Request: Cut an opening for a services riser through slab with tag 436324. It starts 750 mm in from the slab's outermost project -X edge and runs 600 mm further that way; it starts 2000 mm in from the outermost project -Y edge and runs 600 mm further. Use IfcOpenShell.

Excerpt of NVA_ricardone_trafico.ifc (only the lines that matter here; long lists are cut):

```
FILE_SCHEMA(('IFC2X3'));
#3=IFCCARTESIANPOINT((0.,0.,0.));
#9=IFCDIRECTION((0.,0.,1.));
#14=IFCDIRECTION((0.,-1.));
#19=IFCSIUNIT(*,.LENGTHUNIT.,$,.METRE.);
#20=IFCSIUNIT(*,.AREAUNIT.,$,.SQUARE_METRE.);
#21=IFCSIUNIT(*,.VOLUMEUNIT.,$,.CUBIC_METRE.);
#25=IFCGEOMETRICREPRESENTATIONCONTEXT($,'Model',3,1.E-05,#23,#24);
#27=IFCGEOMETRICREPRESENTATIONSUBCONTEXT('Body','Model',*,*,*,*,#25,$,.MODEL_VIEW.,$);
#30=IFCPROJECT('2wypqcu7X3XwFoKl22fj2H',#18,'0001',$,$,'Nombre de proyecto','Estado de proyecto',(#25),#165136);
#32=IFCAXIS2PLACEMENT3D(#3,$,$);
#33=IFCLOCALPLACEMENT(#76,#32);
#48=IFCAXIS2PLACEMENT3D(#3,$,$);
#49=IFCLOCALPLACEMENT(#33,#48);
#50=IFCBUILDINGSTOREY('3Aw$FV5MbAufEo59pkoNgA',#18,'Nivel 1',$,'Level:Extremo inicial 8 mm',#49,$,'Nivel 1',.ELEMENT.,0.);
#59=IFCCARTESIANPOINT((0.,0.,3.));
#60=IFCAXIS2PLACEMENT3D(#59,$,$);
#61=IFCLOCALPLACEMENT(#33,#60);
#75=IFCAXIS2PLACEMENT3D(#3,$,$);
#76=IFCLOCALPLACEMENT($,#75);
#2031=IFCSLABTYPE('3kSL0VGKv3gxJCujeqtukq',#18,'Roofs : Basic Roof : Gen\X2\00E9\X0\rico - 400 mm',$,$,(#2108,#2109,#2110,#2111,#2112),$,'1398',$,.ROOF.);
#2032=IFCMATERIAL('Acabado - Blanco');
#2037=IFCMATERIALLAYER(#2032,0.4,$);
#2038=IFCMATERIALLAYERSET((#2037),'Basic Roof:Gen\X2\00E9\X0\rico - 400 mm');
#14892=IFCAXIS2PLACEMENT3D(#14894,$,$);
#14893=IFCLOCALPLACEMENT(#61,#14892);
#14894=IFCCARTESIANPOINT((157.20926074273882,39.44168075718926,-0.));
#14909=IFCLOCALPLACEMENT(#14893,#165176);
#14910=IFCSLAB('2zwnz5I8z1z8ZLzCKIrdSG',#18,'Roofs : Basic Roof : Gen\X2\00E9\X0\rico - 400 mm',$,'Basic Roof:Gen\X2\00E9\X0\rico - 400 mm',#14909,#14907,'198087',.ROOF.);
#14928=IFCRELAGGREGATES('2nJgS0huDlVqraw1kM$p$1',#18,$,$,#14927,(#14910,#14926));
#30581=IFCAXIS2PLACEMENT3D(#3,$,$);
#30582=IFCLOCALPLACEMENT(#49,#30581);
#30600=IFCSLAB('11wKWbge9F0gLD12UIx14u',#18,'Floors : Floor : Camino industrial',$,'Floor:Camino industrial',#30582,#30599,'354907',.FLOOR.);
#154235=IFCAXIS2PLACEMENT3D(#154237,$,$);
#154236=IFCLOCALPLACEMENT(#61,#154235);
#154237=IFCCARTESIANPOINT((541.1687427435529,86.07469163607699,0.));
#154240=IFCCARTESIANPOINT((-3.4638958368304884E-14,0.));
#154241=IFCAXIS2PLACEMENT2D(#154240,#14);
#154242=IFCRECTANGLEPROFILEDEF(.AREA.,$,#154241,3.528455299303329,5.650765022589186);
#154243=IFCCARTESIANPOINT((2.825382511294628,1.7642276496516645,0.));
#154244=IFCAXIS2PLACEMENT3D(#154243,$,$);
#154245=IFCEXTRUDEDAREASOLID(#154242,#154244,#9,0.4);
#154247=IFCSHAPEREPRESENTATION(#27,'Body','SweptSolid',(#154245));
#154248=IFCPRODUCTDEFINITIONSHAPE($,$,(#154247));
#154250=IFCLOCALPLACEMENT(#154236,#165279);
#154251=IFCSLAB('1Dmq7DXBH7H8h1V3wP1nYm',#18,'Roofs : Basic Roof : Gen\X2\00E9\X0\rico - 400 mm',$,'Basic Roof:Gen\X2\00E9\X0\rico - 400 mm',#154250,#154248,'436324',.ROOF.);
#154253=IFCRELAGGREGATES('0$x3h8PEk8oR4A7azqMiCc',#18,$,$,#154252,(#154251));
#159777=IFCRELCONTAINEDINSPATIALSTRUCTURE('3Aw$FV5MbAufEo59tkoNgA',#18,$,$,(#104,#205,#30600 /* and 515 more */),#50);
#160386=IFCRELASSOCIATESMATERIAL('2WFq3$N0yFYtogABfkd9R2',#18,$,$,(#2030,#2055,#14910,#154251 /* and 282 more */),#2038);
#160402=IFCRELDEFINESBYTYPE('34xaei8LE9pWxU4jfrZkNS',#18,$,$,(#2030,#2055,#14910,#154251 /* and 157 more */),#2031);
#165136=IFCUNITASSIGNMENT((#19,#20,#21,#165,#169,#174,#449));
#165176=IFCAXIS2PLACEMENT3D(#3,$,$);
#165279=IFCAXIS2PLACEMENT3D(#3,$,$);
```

```python
import numpy as np
import ifcopenshell
import ifcopenshell.api.feature
import ifcopenshell.api.geometry
import ifcopenshell.api.root
import ifcopenshell.geom
import ifcopenshell.util.placement
import ifcopenshell.util.representation
import ifcopenshell.util.shape
import ifcopenshell.util.unit

model = ifcopenshell.open("NVA_ricardone_trafico.ifc")
unit_scale = ifcopenshell.util.unit.calculate_unit_scale(model)
settings = ifcopenshell.geom.settings()


def volume(element):
    """Net volume in cubic metres, openings subtracted."""
    shape = ifcopenshell.geom.create_shape(settings, element)
    return ifcopenshell.util.shape.get_volume(shape.geometry)


slab = model.by_guid("1Dmq7DXBH7H8h1V3wP1nYm")
before = volume(slab)

# Extent in the slab's own axes, in metres. The edges named are its -X and -Y sides.
slab_shape = ifcopenshell.geom.create_shape(settings, slab)
vertices = ifcopenshell.util.shape.get_vertices(slab_shape.geometry)
x_min, y_min, bottom = vertices.min(axis=0)
top = vertices[:, 2].max()

opening = ifcopenshell.api.root.create_entity(model, ifc_class="IfcOpeningElement", name="Services riser opening")
context = ifcopenshell.util.representation.get_context(model, "Model", "Body", "MODEL_VIEW")
width, depth = 0.6, 0.6
outline = [(0.0, 0.0), (width, 0.0), (width, depth), (0.0, depth), (0.0, 0.0)]
# Overshoot both faces by 50 mm so the cut is clean.
shape = ifcopenshell.api.geometry.add_slab_representation(
    model, context=context, depth=top - bottom + 0.1, polyline=outline
)
ifcopenshell.api.geometry.assign_representation(model, product=opening, representation=shape)

matrix = ifcopenshell.util.placement.get_local_placement(slab.ObjectPlacement)
matrix[:, 3] = matrix @ np.append(np.array([x_min + 0.75, y_min + 2, bottom - 0.05]) / unit_scale, 1.0)
ifcopenshell.api.geometry.edit_object_placement(model, product=opening, matrix=matrix, is_si=False)
ifcopenshell.api.feature.add_feature(model, feature=opening, element=slab)

after = volume(slab)

print(f"slab volume {before:.3f} -> {after:.3f} m3")

model.write("NVA_ricardone_trafico-out.ifc")
```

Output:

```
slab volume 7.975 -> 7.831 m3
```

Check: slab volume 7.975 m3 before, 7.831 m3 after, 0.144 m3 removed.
